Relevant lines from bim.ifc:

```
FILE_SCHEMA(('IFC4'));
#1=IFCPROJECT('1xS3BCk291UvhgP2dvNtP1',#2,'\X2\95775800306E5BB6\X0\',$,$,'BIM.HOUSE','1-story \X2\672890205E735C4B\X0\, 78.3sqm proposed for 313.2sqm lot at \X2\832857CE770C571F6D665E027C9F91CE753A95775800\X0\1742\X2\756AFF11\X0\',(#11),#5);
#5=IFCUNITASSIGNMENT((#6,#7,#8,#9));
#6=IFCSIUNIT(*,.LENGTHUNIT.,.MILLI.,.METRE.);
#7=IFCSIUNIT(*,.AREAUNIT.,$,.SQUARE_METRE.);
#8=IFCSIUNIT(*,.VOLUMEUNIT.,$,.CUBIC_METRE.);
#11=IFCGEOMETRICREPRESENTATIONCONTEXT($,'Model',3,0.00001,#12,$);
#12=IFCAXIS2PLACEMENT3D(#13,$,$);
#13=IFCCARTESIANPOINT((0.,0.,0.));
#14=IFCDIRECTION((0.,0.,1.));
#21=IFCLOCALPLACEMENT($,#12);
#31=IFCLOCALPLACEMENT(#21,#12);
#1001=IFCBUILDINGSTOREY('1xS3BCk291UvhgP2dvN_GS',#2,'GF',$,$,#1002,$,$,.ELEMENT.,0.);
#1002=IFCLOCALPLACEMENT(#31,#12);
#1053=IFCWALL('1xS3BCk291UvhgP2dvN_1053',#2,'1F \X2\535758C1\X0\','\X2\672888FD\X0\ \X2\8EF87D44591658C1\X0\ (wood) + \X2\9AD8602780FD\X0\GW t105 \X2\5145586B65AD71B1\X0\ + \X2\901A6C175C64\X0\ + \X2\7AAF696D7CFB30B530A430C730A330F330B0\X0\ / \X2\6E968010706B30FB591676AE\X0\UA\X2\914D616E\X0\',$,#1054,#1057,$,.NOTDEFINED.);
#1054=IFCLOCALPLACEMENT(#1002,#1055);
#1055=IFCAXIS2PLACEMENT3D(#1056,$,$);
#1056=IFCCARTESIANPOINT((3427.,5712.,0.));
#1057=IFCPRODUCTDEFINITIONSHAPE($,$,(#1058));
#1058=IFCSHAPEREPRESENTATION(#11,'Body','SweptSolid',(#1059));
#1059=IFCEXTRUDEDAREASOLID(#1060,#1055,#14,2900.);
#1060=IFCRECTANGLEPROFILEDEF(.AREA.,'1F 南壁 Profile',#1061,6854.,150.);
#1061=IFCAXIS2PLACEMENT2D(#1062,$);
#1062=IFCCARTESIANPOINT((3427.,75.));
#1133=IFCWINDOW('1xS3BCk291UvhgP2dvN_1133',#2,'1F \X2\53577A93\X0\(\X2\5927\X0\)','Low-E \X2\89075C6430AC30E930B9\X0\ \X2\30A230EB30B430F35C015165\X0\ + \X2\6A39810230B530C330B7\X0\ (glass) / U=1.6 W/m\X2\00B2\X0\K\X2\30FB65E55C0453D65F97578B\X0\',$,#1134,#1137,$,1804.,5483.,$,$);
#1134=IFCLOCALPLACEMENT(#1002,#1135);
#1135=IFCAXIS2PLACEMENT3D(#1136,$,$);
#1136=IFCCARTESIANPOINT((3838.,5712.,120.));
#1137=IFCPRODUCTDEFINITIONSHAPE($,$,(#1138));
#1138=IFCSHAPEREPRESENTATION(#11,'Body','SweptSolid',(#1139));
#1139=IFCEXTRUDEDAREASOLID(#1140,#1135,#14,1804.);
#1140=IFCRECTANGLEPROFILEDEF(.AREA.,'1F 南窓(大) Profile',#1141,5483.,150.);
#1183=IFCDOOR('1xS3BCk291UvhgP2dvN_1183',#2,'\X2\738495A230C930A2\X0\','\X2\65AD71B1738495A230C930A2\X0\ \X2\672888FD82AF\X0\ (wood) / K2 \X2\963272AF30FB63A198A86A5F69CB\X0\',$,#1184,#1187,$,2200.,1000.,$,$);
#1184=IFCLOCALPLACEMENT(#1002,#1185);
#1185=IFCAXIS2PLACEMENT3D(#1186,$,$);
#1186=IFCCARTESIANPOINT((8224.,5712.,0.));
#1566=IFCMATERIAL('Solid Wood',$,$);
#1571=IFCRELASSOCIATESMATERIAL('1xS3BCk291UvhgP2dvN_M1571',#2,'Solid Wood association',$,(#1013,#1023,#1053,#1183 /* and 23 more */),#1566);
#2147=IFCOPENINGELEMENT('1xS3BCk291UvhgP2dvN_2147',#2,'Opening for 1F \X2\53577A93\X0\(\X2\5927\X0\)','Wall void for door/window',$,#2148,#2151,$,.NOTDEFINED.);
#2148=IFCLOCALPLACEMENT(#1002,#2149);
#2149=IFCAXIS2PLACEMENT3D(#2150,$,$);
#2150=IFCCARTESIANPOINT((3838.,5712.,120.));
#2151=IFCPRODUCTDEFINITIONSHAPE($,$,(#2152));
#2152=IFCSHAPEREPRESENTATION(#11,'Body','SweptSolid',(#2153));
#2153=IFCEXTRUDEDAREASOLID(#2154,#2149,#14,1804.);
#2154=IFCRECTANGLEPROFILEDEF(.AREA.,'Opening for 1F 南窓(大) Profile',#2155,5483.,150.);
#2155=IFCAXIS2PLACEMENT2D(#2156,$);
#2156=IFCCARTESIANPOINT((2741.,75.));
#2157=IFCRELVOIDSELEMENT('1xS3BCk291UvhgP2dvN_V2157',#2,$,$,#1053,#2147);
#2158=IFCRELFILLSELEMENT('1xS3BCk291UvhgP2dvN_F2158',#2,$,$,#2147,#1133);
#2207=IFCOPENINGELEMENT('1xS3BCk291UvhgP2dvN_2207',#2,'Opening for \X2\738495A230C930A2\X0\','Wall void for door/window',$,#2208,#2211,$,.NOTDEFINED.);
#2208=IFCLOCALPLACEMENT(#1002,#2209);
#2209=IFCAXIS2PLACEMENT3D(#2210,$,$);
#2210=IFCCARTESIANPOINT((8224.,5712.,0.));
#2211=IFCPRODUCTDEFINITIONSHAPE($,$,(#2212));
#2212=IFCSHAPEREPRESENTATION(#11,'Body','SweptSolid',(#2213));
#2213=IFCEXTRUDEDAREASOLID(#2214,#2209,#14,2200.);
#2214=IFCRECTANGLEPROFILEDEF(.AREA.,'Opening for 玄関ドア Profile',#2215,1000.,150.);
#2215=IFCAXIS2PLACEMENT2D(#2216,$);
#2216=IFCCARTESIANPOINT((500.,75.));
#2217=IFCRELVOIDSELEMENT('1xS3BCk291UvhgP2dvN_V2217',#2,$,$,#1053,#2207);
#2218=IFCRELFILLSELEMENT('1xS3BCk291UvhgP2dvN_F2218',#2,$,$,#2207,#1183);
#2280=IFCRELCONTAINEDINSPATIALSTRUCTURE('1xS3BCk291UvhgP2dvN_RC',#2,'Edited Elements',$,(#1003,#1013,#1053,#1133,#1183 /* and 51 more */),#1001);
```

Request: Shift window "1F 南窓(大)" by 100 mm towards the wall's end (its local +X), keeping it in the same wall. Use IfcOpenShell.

```python
import ifcopenshell
import ifcopenshell.api.geometry
import ifcopenshell.util.placement
import ifcopenshell.util.unit

model = ifcopenshell.open("bim.ifc")
unit_scale = ifcopenshell.util.unit.calculate_unit_scale(model)

window = model.by_guid("1xS3BCk291UvhgP2dvN_1133")
opening = window.FillsVoids[0].RelatingOpeningElement
wall = opening.VoidsElements[0].RelatingBuildingElement

wall_matrix = ifcopenshell.util.placement.get_local_placement(wall.ObjectPlacement)
shift = wall_matrix[:3, 0] * 0.1 / unit_scale
before = ifcopenshell.util.placement.get_local_placement(window.ObjectPlacement)[:3, 3].copy()

# The window is not placed relative to its opening, so move both.
for product in (opening, window):
    matrix = ifcopenshell.util.placement.get_local_placement(product.ObjectPlacement)
    matrix[:3, 3] += shift
    ifcopenshell.api.geometry.edit_object_placement(model, product=product, matrix=matrix, is_si=False)

after = ifcopenshell.util.placement.get_local_placement(window.ObjectPlacement)[:3, 3]
print("window moved by", (after - before).round(3) + 0.0)

model.write("bim_updated.ifc")
```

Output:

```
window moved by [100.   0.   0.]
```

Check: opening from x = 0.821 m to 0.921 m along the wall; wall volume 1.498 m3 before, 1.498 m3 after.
